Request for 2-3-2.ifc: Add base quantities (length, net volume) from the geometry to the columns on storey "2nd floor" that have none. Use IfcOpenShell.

First a look at what the model holds.

```python
import ifcopenshell
import ifcopenshell.util.element
import ifcopenshell.util.unit

model = ifcopenshell.open("2-3-2.ifc")
print(model.schema)
for unit_type in ("LENGTHUNIT", "AREAUNIT", "VOLUMEUNIT"):
    print(unit_type, ifcopenshell.util.unit.calculate_unit_scale(model, unit_type))
storey = next(s for s in model.by_type("IfcBuildingStorey") if s.Name == "2nd floor")
columns = [e for e in ifcopenshell.util.element.get_decomposition(storey) if e.is_a("IfcColumn")]
for e in sorted(columns, key=lambda e: e.id()):
    print(e.id(), e.is_a(), e.Name, list(ifcopenshell.util.element.get_psets(e, qtos_only=True)), sep=" | ")
```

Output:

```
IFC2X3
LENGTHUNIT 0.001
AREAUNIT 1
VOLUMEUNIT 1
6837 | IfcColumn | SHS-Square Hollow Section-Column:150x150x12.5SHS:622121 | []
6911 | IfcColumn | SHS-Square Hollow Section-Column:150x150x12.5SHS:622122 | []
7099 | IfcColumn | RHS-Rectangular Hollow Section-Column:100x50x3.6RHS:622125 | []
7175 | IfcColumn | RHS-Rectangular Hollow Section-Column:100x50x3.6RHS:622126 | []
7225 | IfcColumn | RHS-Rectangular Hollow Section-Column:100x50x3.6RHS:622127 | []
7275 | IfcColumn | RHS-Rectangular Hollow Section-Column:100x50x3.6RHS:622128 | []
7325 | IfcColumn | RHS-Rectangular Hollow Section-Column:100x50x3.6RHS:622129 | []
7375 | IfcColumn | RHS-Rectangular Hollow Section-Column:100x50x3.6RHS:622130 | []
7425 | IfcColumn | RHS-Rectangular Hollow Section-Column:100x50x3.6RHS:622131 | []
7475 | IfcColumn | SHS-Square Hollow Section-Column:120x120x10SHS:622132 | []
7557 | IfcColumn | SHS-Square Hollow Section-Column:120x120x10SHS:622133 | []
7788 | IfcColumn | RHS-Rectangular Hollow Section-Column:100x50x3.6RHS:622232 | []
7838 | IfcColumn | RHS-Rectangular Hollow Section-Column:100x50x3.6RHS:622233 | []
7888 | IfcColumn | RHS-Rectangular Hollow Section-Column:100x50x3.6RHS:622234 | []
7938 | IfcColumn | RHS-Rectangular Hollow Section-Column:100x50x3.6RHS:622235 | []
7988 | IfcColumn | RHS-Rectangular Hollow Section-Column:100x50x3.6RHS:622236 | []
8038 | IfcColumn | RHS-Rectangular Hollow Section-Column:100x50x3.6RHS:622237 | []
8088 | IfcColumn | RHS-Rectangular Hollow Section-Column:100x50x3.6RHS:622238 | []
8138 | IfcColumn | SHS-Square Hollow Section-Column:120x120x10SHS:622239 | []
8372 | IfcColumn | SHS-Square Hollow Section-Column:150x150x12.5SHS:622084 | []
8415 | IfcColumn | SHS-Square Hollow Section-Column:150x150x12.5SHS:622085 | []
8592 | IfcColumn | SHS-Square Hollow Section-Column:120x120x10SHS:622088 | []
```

```python
import ifcopenshell
import ifcopenshell.api.pset
import ifcopenshell.geom
import ifcopenshell.util.element
import ifcopenshell.util.shape
import ifcopenshell.util.unit

model = ifcopenshell.open("2-3-2.ifc")
unit_scale = ifcopenshell.util.unit.calculate_unit_scale(model)
volume_scale = ifcopenshell.util.unit.calculate_unit_scale(model, "VOLUMEUNIT")
settings = ifcopenshell.geom.settings()

storey = next(s for s in model.by_type("IfcBuildingStorey") if s.Name == "2nd floor")
columns = [e for e in ifcopenshell.util.element.get_decomposition(storey) if e.is_a("IfcColumn")]

for e in sorted(columns, key=lambda e: e.id()):
    if ifcopenshell.util.element.get_psets(e, qtos_only=True, should_inherit=False):
        continue
    # Geometry comes back in metres, in the element's own axes.
    shape = ifcopenshell.geom.create_shape(settings, e)
    values = {
        "Length": ifcopenshell.util.shape.get_z(shape.geometry) / unit_scale,
        "NetVolume": ifcopenshell.util.shape.get_volume(shape.geometry) / volume_scale,
    }
    qto = ifcopenshell.api.pset.add_qto(model, product=e, name="BaseQuantities")
    ifcopenshell.api.pset.edit_qto(model, qto=qto, properties=values)
    print(e.id(), {k: round(v, 3) for k, v in values.items()})

model.write("2-3-2-out.ifc")
```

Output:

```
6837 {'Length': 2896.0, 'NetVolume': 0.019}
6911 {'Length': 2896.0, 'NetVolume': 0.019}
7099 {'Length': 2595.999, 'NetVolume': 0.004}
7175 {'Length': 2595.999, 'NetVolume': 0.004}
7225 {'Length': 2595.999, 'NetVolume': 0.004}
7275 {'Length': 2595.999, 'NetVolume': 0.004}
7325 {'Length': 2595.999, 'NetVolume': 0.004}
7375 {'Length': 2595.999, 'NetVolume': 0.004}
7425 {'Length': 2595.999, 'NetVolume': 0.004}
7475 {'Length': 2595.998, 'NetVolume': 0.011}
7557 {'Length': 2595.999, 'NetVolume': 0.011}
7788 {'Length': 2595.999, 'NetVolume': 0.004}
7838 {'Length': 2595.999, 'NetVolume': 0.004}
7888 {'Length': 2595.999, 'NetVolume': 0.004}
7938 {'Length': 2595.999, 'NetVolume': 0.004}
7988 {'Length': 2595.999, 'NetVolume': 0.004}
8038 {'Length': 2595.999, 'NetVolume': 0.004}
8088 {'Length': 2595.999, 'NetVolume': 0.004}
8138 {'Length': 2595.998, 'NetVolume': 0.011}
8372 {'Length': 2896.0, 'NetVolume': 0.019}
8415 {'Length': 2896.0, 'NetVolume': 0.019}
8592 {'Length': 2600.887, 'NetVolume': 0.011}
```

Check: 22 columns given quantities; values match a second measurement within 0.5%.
